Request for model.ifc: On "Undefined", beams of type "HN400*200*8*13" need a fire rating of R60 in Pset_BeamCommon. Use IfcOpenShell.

First a look at what the model holds.

```python
import ifcopenshell
import ifcopenshell.util.element

model = ifcopenshell.open("model.ifc")
print(model.schema)
storey = next(s for s in model.by_type("IfcBuildingStorey") if s.Name == "Undefined")
beams = [e for e in ifcopenshell.util.element.get_decomposition(storey) if e.is_a("IfcBeam")]
seen = {}
for e in beams:
    element_type = ifcopenshell.util.element.get_type(e)
    key = (element_type.Name if element_type != e and element_type else None, ifcopenshell.util.element.get_pset(e, "Pset_BeamCommon", "FireRating"))
    seen[key] = seen.get(key, 0) + 1
for (name, value), count in sorted(seen.items(), key=str):
    print(count, "x", name, "|", value)
```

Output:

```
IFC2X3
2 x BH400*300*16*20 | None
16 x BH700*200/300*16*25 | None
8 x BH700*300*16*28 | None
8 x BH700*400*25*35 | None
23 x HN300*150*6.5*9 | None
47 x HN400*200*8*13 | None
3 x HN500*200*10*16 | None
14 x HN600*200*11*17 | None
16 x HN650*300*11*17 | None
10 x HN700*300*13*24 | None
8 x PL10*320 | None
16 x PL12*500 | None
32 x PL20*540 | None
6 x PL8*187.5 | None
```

```python
import ifcopenshell
import ifcopenshell.api.pset
import ifcopenshell.util.element

model = ifcopenshell.open("model.ifc")

storey = next(s for s in model.by_type("IfcBuildingStorey") if s.Name == "Undefined")
beams = [e for e in ifcopenshell.util.element.get_decomposition(storey) if e.is_a("IfcBeam")]

count = 0
for e in beams:
    element_type = ifcopenshell.util.element.get_type(e)
    if element_type in (None, e) or element_type.Name != "HN400*200*8*13":
        continue
    # add_pset returns the element's existing set when there is one.
    pset = ifcopenshell.api.pset.add_pset(model, product=e, name="Pset_BeamCommon")
    ifcopenshell.api.pset.edit_pset(model, pset=pset, properties={"FireRating": "R60"})
    count += 1

print(count, "beams updated")

model.write("model_edited.ifc")
```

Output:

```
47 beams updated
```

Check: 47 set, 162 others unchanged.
